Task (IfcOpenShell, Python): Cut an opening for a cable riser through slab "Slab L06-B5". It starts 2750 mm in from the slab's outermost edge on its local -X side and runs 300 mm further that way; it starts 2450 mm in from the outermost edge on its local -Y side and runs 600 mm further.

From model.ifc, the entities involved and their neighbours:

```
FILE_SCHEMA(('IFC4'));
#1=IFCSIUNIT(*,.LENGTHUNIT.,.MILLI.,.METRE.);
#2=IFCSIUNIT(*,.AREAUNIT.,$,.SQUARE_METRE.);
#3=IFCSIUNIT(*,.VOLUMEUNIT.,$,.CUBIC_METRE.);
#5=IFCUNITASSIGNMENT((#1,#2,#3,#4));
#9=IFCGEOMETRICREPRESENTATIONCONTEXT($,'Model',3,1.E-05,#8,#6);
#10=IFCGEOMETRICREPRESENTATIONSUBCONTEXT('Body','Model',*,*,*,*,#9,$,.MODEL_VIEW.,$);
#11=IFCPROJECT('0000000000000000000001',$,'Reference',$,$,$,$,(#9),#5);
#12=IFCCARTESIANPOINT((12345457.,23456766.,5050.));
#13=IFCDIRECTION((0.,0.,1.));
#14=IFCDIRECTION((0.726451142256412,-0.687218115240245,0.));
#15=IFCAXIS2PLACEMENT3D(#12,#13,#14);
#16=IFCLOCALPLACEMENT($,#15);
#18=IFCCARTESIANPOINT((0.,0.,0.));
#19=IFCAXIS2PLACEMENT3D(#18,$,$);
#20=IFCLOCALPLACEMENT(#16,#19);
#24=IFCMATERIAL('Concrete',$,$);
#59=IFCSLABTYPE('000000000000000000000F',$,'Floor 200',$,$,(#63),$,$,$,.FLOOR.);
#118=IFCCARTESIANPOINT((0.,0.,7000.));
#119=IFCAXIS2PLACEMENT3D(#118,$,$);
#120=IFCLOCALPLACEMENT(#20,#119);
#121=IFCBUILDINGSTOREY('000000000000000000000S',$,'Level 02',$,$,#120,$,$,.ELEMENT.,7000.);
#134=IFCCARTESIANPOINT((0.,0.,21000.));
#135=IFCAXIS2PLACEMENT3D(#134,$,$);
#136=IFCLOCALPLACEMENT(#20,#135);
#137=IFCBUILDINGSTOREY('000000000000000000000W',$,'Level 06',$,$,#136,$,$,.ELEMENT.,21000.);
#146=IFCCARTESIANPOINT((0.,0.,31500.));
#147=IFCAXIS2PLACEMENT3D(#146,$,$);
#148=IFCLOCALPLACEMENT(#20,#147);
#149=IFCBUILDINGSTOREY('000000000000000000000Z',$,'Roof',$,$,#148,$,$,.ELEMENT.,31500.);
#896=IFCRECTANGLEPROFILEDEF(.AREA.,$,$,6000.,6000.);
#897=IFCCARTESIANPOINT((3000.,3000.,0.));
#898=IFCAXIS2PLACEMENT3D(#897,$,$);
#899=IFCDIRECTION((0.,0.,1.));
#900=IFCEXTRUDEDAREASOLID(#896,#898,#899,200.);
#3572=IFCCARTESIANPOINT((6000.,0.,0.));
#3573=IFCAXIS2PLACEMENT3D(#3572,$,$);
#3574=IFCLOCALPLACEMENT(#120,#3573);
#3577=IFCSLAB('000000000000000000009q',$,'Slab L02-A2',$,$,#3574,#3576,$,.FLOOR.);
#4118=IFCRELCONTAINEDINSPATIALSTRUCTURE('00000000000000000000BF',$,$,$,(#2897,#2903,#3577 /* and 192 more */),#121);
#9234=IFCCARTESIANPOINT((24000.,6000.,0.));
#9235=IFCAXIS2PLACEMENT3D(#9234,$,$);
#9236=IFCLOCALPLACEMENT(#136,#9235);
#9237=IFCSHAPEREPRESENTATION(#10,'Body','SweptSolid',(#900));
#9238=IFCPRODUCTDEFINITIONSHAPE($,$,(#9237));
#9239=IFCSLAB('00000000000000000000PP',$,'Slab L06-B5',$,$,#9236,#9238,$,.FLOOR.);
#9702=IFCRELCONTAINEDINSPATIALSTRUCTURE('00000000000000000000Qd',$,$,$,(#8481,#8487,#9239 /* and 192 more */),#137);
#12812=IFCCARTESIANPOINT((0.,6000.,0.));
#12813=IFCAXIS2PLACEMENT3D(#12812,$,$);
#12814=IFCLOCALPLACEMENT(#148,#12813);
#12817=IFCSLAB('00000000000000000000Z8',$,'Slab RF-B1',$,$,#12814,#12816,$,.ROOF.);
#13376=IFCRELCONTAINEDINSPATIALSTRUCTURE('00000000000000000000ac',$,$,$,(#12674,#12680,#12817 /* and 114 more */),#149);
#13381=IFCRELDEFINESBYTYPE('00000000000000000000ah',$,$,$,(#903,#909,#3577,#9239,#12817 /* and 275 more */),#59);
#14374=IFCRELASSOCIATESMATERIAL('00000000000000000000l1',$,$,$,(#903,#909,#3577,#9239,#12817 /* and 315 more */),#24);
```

```python
import numpy as np
import ifcopenshell
import ifcopenshell.api.feature
import ifcopenshell.api.geometry
import ifcopenshell.api.root
import ifcopenshell.geom
import ifcopenshell.util.placement
import ifcopenshell.util.representation
import ifcopenshell.util.shape
import ifcopenshell.util.unit

model = ifcopenshell.open("model.ifc")
unit_scale = ifcopenshell.util.unit.calculate_unit_scale(model)
settings = ifcopenshell.geom.settings()


def volume(element):
    """Net volume in cubic metres, openings subtracted."""
    shape = ifcopenshell.geom.create_shape(settings, element)
    return ifcopenshell.util.shape.get_volume(shape.geometry)


slab = model.by_id(9239)
before = volume(slab)

# Extent in the slab's own axes, in metres. The edges named are its -X and -Y sides.
slab_shape = ifcopenshell.geom.create_shape(settings, slab)
vertices = ifcopenshell.util.shape.get_vertices(slab_shape.geometry)
x_min, y_min, bottom = vertices.min(axis=0)
top = vertices[:, 2].max()

opening = ifcopenshell.api.root.create_entity(model, ifc_class="IfcOpeningElement", name="Cable riser opening", predefined_type="OPENING")
context = ifcopenshell.util.representation.get_context(model, "Model", "Body", "MODEL_VIEW")
width, depth = 0.3, 0.6
outline = [(0.0, 0.0), (width, 0.0), (width, depth), (0.0, depth), (0.0, 0.0)]
# Overshoot both faces by 50 mm so the cut is clean.
shape = ifcopenshell.api.geometry.add_slab_representation(
    model, context=context, depth=top - bottom + 0.1, polyline=outline
)
ifcopenshell.api.geometry.assign_representation(model, product=opening, representation=shape)

matrix = ifcopenshell.util.placement.get_local_placement(slab.ObjectPlacement)
matrix[:, 3] = matrix @ np.append(np.array([x_min + 2.75, y_min + 2.45, bottom - 0.05]) / unit_scale, 1.0)
ifcopenshell.api.geometry.edit_object_placement(model, product=opening, matrix=matrix, is_si=False)
ifcopenshell.api.feature.add_feature(model, feature=opening, element=slab)

after = volume(slab)

print(f"slab volume {before:.3f} -> {after:.3f} m3")

model.write("model_updated.ifc")
```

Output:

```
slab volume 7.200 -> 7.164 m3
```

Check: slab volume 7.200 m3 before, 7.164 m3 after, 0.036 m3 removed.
